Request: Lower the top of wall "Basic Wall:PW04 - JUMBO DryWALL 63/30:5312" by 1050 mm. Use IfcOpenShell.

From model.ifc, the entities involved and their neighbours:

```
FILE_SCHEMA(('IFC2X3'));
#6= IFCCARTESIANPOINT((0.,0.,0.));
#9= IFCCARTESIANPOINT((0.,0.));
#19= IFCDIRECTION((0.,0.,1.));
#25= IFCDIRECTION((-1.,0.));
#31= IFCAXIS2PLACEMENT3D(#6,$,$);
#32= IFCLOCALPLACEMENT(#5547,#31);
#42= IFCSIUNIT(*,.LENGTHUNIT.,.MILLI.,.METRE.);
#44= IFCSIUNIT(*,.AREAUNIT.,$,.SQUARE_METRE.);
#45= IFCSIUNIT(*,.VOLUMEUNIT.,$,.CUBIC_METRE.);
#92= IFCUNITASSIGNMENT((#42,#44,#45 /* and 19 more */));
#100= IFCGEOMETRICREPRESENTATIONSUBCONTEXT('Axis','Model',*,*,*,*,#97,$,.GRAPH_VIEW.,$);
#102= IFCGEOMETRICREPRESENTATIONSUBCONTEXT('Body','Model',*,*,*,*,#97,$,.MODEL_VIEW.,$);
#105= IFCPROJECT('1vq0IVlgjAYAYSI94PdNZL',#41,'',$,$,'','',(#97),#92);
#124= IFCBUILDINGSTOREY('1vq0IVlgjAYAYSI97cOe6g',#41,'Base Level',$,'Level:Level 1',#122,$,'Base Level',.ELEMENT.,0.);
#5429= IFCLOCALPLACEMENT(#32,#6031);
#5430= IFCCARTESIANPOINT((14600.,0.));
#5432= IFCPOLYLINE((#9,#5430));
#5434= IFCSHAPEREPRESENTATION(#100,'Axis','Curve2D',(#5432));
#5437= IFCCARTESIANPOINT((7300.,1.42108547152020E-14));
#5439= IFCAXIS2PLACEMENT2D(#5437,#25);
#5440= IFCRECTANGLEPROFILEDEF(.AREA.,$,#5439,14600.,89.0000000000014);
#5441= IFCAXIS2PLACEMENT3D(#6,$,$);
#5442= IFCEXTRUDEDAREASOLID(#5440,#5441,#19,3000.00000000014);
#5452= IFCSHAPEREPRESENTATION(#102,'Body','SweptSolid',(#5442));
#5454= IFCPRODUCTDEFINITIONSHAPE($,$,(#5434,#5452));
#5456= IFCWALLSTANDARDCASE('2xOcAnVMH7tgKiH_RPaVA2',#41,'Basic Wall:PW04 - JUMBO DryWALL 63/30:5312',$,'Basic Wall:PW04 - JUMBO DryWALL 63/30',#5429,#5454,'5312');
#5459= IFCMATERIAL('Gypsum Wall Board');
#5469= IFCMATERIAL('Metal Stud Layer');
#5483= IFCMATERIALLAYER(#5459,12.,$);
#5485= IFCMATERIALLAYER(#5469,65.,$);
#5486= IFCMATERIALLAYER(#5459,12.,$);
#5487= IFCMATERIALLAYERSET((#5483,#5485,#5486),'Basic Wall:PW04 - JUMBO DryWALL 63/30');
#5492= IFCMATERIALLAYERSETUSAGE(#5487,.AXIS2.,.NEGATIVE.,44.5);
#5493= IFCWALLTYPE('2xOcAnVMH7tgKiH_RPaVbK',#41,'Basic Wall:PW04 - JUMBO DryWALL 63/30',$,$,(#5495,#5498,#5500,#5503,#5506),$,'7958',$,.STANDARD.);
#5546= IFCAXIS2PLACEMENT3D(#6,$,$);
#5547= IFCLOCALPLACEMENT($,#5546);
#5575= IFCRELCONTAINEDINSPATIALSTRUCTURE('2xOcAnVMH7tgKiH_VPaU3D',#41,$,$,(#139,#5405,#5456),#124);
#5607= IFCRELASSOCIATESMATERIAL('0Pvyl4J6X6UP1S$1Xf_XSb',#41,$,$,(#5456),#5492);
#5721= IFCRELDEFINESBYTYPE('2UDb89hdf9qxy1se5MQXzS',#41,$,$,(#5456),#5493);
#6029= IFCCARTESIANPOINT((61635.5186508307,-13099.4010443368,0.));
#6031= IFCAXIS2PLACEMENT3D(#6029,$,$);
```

```python
import ifcopenshell
import ifcopenshell.geom
import ifcopenshell.util.representation
import ifcopenshell.util.shape
import ifcopenshell.util.unit

model = ifcopenshell.open("model.ifc")
unit_scale = ifcopenshell.util.unit.calculate_unit_scale(model)
settings = ifcopenshell.geom.settings()


def volume(element):
    """Net volume in cubic metres, openings subtracted."""
    shape = ifcopenshell.geom.create_shape(settings, element)
    return ifcopenshell.util.shape.get_volume(shape.geometry)


wall = model.by_guid("2xOcAnVMH7tgKiH_RPaVA2")
before = volume(wall)

body = ifcopenshell.util.representation.get_representation(wall, "Model", "Body")
solid = body.Items[0]
old_height = solid.Depth
solid.Depth -= 1.05 / unit_scale
after = volume(wall)

print(f"height {old_height:g} -> {solid.Depth:g}, volume {before:.3f} -> {after:.3f} m3")

model.write("model_rev.ifc")
```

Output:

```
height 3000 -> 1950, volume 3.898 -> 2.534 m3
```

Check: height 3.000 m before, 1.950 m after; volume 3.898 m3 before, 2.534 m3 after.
